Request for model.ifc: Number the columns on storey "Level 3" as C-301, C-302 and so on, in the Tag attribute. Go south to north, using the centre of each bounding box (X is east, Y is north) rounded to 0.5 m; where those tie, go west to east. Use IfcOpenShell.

First a look at what the model holds.

```python
import ifcopenshell
import ifcopenshell.util.element
import ifcopenshell.util.placement

model = ifcopenshell.open("model.ifc")
print(model.schema)
storey = next(s for s in model.by_type("IfcBuildingStorey") if s.Name == "Level 3")
columns = [e for e in ifcopenshell.util.element.get_decomposition(storey) if e.is_a("IfcColumn")]
for e in sorted(columns, key=lambda e: e.id()):
    origin = ifcopenshell.util.placement.get_local_placement(e.ObjectPlacement)[:3, 3]
    print(e.id(), e.Tag, e.Name, origin.round(2) + 0.0, sep=" | ")
```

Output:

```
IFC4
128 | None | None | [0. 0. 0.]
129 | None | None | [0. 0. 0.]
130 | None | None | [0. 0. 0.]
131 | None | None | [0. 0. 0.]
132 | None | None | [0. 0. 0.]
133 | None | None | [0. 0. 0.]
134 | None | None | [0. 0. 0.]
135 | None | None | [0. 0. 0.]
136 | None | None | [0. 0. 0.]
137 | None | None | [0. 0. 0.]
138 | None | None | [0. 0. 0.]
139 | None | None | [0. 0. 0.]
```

```python
import ifcopenshell
import ifcopenshell.geom
import ifcopenshell.util.element
import ifcopenshell.util.shape

model = ifcopenshell.open("model.ifc")
settings = ifcopenshell.geom.settings()
settings.set("use-world-coords", True)


def centre(element):
    shape = ifcopenshell.geom.create_shape(settings, element)
    return ifcopenshell.util.shape.get_bbox_centroid(shape.geometry)


storey = next(s for s in model.by_type("IfcBuildingStorey") if s.Name == "Level 3")
columns = [e for e in ifcopenshell.util.element.get_decomposition(storey) if e.is_a("IfcColumn")]

# Insertion points can sit at a corner or the storey origin, so sort by the geometry (in metres).
centres = {e: centre(e) for e in columns}
columns.sort(key=lambda e: (round(centres[e][1] / 0.5), centres[e][0]))

for i, e in enumerate(columns, start=1):
    number = f"C-3{i:02d}"
    e.Tag = number
    print(e.id(), number)

model.write("model_updated.ifc")
```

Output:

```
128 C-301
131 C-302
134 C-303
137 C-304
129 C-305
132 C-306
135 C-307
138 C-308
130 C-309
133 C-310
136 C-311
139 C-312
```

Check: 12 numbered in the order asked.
